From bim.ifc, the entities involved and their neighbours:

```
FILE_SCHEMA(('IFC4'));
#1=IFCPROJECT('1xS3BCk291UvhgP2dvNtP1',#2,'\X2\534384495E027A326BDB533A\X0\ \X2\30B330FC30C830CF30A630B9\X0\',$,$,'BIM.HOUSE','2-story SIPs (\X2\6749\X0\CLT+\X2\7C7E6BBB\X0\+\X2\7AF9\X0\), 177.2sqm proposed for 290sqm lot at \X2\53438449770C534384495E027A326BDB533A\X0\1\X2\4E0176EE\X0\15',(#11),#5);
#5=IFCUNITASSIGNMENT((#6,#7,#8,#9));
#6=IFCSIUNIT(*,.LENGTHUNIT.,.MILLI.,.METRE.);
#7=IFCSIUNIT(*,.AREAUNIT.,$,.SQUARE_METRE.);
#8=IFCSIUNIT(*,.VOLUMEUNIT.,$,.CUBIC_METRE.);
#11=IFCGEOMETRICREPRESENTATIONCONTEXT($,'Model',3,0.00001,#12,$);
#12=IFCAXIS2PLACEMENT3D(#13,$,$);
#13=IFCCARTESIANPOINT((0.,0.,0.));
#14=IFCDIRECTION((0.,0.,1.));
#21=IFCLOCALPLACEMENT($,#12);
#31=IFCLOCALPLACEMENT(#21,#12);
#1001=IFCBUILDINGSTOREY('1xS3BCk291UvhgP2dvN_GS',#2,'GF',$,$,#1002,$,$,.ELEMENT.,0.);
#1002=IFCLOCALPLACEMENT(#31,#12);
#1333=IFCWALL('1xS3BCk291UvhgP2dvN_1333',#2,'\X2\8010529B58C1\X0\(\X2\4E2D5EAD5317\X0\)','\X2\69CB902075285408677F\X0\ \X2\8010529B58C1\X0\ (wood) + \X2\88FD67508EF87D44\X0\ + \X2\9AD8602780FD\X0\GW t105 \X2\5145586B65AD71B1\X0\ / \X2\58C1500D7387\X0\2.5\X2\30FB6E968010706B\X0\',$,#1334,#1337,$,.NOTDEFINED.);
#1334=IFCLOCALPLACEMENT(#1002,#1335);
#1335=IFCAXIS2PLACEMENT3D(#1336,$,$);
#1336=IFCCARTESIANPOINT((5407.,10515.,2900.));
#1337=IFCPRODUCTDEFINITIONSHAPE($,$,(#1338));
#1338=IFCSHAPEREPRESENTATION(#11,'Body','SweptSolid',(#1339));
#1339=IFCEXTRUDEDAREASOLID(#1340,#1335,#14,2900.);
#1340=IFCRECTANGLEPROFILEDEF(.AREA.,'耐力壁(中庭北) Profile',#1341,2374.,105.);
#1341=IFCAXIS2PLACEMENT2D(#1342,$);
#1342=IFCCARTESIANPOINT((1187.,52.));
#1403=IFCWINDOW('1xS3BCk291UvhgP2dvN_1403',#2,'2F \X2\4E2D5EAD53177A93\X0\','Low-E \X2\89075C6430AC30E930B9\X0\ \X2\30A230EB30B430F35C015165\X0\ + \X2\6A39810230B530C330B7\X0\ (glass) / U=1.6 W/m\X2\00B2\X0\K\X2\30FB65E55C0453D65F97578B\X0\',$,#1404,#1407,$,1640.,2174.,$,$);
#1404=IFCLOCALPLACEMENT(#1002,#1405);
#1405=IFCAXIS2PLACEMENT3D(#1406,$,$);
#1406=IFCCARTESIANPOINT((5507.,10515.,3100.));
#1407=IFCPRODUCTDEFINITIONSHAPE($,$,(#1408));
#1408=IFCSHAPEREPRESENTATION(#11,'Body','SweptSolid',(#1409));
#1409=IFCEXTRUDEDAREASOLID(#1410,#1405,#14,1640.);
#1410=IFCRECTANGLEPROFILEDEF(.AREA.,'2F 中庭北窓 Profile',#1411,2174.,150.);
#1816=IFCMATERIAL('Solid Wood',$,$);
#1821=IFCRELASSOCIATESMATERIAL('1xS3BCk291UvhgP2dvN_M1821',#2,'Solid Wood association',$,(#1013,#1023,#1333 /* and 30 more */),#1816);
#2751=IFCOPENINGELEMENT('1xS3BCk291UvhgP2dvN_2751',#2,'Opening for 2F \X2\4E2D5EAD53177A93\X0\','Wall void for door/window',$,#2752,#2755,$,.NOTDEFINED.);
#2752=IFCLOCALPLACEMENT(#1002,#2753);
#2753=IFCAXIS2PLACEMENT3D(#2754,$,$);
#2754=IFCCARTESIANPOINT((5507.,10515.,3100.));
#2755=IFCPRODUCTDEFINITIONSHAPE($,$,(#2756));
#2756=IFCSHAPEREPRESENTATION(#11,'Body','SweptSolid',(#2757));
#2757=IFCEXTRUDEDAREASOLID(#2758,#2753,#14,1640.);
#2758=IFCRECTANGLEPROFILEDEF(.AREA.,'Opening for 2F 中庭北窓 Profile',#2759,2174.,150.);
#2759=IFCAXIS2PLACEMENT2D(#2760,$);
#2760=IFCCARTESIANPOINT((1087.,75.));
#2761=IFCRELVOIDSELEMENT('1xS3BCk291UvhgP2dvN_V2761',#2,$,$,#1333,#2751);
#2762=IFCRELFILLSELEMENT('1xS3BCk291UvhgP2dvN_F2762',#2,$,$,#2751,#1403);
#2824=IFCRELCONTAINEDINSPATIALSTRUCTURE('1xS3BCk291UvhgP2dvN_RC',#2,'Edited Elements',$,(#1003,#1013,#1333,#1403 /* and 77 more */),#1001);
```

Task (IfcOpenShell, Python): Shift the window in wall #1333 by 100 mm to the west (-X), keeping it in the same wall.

```python
import ifcopenshell
import ifcopenshell.api.geometry
import ifcopenshell.util.placement
import ifcopenshell.util.unit

model = ifcopenshell.open("bim.ifc")
unit_scale = ifcopenshell.util.unit.calculate_unit_scale(model)

window = model.by_id(1403)
opening = window.FillsVoids[0].RelatingOpeningElement
wall = opening.VoidsElements[0].RelatingBuildingElement

wall_matrix = ifcopenshell.util.placement.get_local_placement(wall.ObjectPlacement)
shift = wall_matrix[:3, 0] * -0.1 / unit_scale
before = ifcopenshell.util.placement.get_local_placement(window.ObjectPlacement)[:3, 3].copy()

# The window is not placed relative to its opening, so move both.
for product in (opening, window):
    matrix = ifcopenshell.util.placement.get_local_placement(product.ObjectPlacement)
    matrix[:3, 3] += shift
    ifcopenshell.api.geometry.edit_object_placement(model, product=product, matrix=matrix, is_si=False)

after = ifcopenshell.util.placement.get_local_placement(window.ObjectPlacement)[:3, 3]
print("window moved by", (after - before).round(3) + 0.0)

model.write("bim_rev.ifc")
```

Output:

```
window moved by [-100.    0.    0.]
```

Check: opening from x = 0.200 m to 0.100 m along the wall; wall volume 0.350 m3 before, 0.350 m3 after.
